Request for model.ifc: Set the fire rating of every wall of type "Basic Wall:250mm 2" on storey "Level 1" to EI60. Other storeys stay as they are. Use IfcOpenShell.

First a look at what the model holds.

```python
import ifcopenshell
import ifcopenshell.util.element

model = ifcopenshell.open("model.ifc")
print(model.schema)
storey = next(s for s in model.by_type("IfcBuildingStorey") if s.Name == "Level 1")
walls = [e for e in ifcopenshell.util.element.get_decomposition(storey) if e.is_a("IfcWall")]
seen = {}
for e in walls:
    element_type = ifcopenshell.util.element.get_type(e)
    key = (element_type.Name if element_type != e and element_type else None, ifcopenshell.util.element.get_pset(e, "Pset_WallCommon", "FireRating"))
    seen[key] = seen.get(key, 0) + 1
for (name, value), count in sorted(seen.items(), key=str):
    print(count, "x", name, "|", value)
```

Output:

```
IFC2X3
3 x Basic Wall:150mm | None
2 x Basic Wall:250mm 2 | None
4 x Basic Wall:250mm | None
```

```python
import ifcopenshell
import ifcopenshell.api.pset
import ifcopenshell.util.element

model = ifcopenshell.open("model.ifc")

storey = next(s for s in model.by_type("IfcBuildingStorey") if s.Name == "Level 1")
walls = [e for e in ifcopenshell.util.element.get_decomposition(storey) if e.is_a("IfcWall")]

count = 0
for e in walls:
    element_type = ifcopenshell.util.element.get_type(e)
    if element_type in (None, e) or element_type.Name != "Basic Wall:250mm 2":
        continue
    # add_pset returns the element's existing set when there is one.
    pset = ifcopenshell.api.pset.add_pset(model, product=e, name="Pset_WallCommon")
    ifcopenshell.api.pset.edit_pset(model, pset=pset, properties={"FireRating": "EI60"})
    count += 1

print(count, "walls updated")

model.write("model-out.ifc")
```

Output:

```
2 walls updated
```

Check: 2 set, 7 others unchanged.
